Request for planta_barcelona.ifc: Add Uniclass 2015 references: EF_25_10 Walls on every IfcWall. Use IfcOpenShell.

First a look at what the model holds.

```python
import ifcopenshell

model = ifcopenshell.open("planta_barcelona.ifc")
print(model.schema)
print("classifications:", [c.Name for c in model.by_type("IfcClassification")])
for ifc_class in ("IfcDoor", "IfcRoof", "IfcStair", "IfcWall", "IfcWindow"):
    print(ifc_class, len(model.by_type(ifc_class)))
```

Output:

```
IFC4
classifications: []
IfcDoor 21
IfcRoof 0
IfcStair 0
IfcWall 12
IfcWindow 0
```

```python
import ifcopenshell
import ifcopenshell.api.classification

model = ifcopenshell.open("planta_barcelona.ifc")

system = ifcopenshell.api.classification.add_classification(model, classification="Uniclass 2015")

codes = {
    "IfcWall": ("EF_25_10", "Walls"),
}
for ifc_class, (code, name) in codes.items():
    products = model.by_type(ifc_class)
    ifcopenshell.api.classification.add_reference(
        model, products=products, classification=system, identification=code, name=name
    )
    print(code, len(products))

model.write("planta_barcelona_rev.ifc")
```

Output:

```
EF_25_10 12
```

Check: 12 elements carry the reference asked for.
